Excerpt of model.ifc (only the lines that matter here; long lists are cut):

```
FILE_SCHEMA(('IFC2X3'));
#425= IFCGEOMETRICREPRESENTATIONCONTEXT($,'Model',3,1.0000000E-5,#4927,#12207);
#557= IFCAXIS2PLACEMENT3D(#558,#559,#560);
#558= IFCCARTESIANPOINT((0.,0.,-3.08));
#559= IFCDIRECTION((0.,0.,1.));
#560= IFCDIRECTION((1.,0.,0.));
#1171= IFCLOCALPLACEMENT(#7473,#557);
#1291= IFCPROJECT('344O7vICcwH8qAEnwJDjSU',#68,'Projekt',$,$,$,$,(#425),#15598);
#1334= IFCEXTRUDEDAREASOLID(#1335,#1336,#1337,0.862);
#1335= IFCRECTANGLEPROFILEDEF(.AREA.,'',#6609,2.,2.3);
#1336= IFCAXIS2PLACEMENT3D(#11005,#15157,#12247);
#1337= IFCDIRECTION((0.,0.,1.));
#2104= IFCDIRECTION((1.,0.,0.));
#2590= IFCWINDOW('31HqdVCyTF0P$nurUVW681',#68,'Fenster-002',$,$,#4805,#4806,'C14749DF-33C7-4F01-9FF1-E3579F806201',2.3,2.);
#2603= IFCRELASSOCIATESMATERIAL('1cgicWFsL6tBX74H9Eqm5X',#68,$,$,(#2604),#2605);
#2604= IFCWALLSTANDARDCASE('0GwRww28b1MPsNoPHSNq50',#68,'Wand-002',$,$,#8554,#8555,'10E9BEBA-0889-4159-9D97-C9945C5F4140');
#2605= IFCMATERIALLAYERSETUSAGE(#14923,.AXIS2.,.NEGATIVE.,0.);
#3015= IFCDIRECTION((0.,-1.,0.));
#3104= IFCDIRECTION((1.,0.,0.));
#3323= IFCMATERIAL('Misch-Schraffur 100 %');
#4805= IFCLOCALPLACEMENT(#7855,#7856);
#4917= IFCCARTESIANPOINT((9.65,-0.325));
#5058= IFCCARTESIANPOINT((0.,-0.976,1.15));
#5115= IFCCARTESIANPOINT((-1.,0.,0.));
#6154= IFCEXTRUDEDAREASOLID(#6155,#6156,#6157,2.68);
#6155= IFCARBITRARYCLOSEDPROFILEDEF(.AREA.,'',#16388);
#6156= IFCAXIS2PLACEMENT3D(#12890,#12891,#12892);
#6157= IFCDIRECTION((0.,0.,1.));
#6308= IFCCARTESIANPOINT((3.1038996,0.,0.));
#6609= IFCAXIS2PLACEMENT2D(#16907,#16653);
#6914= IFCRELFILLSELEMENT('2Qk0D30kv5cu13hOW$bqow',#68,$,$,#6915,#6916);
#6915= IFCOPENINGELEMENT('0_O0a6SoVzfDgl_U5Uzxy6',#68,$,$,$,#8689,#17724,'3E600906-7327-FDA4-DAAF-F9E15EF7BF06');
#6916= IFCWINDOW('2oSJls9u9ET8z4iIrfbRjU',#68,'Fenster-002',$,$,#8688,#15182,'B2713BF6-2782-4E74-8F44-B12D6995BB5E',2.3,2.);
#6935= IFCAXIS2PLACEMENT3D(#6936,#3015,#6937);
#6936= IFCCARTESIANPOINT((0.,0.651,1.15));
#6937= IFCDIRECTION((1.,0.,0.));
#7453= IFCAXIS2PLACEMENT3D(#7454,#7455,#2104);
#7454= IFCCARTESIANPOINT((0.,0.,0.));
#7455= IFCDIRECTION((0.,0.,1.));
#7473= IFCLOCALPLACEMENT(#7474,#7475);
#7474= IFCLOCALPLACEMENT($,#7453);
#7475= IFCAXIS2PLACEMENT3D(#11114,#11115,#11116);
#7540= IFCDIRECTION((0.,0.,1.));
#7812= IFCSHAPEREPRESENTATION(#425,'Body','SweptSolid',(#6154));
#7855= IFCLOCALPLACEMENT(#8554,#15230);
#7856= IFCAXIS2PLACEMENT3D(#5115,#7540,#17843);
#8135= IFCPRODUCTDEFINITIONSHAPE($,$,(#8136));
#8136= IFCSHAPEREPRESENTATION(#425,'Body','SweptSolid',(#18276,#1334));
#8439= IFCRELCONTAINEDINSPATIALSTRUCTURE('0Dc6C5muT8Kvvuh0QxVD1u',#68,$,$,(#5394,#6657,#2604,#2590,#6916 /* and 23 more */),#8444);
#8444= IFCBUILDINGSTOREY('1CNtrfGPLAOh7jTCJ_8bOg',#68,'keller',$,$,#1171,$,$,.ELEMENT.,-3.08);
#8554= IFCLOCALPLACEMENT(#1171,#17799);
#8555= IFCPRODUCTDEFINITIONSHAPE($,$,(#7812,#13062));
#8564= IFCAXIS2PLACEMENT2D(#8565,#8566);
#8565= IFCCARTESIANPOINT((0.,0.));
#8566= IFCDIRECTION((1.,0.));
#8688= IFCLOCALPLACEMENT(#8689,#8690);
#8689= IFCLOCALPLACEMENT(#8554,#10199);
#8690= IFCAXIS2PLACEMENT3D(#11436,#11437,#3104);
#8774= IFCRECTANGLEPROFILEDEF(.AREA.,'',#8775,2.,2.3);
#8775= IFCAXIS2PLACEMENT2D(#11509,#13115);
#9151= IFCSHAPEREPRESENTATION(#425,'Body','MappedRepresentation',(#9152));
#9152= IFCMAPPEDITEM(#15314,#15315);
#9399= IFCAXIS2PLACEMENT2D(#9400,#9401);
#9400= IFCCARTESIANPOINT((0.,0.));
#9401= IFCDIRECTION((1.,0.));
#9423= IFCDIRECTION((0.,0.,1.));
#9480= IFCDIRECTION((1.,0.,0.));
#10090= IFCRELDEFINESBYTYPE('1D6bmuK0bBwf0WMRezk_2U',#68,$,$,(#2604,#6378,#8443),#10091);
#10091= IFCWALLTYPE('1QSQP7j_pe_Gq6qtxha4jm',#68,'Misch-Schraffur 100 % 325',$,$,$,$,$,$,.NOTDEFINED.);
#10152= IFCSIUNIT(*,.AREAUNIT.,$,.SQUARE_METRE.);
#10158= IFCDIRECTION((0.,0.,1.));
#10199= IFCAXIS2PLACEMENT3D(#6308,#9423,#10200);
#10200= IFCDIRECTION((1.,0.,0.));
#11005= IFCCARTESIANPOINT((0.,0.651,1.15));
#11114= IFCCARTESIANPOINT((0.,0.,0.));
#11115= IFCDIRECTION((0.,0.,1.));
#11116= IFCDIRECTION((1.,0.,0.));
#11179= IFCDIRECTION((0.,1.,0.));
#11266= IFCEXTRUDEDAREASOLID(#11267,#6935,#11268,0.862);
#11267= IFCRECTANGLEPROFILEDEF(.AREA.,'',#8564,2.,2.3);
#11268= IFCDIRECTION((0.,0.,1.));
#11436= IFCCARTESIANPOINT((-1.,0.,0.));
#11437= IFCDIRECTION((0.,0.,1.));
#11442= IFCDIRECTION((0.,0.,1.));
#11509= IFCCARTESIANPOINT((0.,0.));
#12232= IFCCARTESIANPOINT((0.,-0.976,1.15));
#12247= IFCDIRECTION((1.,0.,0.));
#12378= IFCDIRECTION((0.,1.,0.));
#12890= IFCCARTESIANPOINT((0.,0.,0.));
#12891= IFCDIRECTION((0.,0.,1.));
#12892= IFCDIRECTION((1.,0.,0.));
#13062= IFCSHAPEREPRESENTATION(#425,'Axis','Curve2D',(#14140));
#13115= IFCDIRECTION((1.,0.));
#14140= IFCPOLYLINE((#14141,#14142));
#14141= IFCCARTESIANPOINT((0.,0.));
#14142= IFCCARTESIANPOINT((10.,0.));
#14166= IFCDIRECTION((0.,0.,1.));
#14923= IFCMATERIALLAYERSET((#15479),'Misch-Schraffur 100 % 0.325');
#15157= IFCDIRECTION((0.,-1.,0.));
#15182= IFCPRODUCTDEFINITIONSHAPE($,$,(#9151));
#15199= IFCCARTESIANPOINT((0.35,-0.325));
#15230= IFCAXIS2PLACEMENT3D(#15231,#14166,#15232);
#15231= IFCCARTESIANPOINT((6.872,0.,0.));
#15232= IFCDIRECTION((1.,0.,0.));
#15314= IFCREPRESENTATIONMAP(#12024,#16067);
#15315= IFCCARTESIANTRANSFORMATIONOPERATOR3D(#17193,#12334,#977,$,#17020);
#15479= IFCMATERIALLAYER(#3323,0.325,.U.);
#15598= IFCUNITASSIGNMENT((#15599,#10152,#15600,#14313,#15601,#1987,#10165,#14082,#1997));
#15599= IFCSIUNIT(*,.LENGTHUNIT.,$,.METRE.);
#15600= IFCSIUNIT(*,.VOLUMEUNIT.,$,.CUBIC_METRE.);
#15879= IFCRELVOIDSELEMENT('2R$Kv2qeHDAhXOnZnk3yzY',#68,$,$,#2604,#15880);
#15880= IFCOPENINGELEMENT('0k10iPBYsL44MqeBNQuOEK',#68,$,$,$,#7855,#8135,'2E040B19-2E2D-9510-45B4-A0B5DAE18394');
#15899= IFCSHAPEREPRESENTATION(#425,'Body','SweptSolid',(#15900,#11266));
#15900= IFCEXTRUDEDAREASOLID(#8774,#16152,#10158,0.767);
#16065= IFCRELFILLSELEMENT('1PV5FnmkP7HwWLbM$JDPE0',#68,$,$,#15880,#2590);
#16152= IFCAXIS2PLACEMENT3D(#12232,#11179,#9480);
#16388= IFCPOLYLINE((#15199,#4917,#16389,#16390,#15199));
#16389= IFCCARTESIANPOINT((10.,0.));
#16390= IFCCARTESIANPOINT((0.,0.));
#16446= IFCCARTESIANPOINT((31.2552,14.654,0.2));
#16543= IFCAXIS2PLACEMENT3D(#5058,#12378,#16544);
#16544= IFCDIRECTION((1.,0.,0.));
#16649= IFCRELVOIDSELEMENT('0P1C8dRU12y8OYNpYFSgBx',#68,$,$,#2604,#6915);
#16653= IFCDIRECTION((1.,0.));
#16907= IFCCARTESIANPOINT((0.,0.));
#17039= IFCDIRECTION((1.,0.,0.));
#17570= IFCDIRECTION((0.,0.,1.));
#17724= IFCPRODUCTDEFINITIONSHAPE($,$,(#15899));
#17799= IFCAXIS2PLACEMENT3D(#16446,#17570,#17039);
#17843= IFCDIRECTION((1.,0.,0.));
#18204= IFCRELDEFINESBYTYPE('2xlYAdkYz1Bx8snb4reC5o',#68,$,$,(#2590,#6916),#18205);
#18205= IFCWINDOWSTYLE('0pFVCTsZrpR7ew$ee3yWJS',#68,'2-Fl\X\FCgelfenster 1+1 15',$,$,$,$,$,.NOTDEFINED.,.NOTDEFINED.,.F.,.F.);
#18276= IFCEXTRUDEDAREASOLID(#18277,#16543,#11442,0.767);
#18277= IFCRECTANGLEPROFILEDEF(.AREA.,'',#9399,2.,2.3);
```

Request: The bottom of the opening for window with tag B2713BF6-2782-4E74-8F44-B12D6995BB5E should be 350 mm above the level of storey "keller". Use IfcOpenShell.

```python
import numpy as np
import ifcopenshell
import ifcopenshell.api.geometry
import ifcopenshell.geom
import ifcopenshell.util.element
import ifcopenshell.util.placement
import ifcopenshell.util.shape
import ifcopenshell.util.unit

model = ifcopenshell.open("model.ifc")
unit_scale = ifcopenshell.util.unit.calculate_unit_scale(model)

window = model.by_id(6916)
opening = window.FillsVoids[0].RelatingOpeningElement
storey = ifcopenshell.util.element.get_container(window, ifc_class="IfcBuildingStorey")
level = ifcopenshell.util.placement.get_local_placement(storey.ObjectPlacement)[2, 3]

# The opening's origin need not be at the sill, so measure its lowest point.
shape = ifcopenshell.geom.create_shape(ifcopenshell.geom.settings(), opening)
bottom = ifcopenshell.util.shape.get_shape_bottom_elevation(shape, shape.geometry) / unit_scale
dz = level + 0.35 / unit_scale - bottom

shift = np.array([0.0, 0.0, dz])
# The window is placed relative to its opening, so it follows when the opening moves.
matrix = ifcopenshell.util.placement.get_local_placement(opening.ObjectPlacement)
matrix[:3, 3] += shift
ifcopenshell.api.geometry.edit_object_placement(
    model, product=opening, matrix=matrix, is_si=False, should_transform_children=True
)

print(f"moved by {dz * unit_scale:+.3f} m")

model.write("model-out.ifc")
```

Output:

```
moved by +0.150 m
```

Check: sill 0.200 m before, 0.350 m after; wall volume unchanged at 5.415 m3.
